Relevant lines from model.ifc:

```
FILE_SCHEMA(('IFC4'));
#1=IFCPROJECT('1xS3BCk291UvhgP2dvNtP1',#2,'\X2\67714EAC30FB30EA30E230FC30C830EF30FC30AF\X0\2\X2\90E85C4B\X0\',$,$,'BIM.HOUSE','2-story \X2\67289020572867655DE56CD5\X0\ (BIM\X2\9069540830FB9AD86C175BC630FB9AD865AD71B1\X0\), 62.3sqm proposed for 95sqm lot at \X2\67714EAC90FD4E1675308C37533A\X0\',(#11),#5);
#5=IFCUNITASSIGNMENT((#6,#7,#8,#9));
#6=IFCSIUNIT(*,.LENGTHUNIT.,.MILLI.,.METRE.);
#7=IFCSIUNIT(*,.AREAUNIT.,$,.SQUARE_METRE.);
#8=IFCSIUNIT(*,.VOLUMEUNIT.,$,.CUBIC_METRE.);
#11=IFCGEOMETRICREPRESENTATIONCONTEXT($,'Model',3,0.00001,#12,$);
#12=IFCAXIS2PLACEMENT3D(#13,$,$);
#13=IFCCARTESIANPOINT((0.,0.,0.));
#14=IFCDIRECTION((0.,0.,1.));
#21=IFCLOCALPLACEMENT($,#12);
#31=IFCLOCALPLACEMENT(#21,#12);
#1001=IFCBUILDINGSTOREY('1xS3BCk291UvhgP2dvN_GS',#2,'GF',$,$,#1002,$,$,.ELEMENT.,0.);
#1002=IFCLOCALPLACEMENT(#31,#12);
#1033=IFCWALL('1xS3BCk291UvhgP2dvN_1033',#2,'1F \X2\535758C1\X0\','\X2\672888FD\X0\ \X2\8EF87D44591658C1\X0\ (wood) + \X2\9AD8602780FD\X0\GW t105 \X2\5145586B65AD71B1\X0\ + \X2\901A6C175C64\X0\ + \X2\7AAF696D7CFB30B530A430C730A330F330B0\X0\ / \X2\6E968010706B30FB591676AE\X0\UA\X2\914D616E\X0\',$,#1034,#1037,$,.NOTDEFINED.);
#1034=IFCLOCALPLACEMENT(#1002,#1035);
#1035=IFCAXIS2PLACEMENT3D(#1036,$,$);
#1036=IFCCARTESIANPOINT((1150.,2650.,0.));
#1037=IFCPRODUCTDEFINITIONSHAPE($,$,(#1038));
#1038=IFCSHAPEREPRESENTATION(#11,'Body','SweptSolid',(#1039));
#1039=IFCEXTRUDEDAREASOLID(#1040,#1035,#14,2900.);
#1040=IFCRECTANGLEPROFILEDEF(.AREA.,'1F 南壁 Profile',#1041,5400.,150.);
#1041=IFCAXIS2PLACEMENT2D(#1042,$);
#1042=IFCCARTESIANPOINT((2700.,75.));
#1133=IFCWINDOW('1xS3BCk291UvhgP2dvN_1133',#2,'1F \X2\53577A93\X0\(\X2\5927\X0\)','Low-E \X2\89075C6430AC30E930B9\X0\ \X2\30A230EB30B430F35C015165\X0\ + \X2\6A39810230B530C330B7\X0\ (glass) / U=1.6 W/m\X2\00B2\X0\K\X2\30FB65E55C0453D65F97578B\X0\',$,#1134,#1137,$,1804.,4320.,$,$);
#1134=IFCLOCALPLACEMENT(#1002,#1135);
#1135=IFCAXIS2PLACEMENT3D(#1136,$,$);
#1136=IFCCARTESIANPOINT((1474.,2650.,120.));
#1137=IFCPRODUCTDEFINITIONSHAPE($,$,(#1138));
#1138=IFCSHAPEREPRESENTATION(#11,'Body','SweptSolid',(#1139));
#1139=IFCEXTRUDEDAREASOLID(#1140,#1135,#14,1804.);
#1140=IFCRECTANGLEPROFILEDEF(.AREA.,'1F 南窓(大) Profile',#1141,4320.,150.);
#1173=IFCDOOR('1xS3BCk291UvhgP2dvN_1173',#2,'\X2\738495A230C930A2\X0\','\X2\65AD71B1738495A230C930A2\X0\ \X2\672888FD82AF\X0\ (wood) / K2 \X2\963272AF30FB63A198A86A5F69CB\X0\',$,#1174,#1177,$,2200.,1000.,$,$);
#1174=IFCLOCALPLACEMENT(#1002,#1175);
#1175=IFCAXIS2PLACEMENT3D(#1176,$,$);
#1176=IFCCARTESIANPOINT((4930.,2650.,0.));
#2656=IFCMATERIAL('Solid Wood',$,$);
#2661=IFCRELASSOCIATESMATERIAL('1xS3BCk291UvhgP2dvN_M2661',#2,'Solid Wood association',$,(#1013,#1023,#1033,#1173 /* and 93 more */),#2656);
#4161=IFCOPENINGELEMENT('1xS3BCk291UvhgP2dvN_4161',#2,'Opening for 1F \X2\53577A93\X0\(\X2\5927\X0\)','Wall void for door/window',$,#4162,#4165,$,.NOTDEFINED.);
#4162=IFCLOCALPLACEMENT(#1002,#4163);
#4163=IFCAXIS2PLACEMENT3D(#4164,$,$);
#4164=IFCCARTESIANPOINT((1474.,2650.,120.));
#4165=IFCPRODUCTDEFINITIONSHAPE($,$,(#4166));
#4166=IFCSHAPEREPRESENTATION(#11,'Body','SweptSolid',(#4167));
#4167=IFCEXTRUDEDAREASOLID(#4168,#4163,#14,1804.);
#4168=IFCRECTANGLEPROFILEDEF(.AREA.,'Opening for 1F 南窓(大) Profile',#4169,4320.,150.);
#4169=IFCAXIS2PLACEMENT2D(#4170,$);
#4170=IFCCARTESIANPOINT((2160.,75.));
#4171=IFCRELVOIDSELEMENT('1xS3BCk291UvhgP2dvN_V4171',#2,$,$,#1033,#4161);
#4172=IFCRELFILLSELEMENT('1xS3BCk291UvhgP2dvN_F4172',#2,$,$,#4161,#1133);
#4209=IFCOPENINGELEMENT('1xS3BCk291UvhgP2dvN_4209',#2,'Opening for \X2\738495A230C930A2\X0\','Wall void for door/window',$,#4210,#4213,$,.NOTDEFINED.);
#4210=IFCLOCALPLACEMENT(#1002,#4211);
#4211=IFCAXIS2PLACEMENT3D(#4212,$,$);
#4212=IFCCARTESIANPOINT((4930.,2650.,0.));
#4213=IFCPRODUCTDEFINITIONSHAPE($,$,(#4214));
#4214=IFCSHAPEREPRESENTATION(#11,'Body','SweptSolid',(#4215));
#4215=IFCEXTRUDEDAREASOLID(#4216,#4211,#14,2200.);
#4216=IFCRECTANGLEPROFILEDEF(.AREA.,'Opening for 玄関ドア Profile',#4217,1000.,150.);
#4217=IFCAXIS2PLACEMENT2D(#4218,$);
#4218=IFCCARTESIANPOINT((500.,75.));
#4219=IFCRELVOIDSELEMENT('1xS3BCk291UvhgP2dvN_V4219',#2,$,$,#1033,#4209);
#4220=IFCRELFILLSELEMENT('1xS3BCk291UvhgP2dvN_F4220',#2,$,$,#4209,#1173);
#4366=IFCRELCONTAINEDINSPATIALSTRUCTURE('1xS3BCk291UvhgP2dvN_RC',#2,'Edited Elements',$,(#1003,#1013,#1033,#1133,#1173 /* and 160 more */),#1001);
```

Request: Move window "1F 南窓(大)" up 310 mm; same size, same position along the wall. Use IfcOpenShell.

```python
import numpy as np
import ifcopenshell
import ifcopenshell.api.geometry
import ifcopenshell.util.placement
import ifcopenshell.util.unit

model = ifcopenshell.open("model.ifc")
unit_scale = ifcopenshell.util.unit.calculate_unit_scale(model)

window = model.by_guid("1xS3BCk291UvhgP2dvN_1133")
opening = window.FillsVoids[0].RelatingOpeningElement
dz = 0.31 / unit_scale

shift = np.array([0.0, 0.0, dz])
# The window is not placed relative to its opening, so move both.
for product in (opening, window):
    matrix = ifcopenshell.util.placement.get_local_placement(product.ObjectPlacement)
    matrix[:3, 3] += shift
    ifcopenshell.api.geometry.edit_object_placement(model, product=product, matrix=matrix, is_si=False)

print(f"moved by {dz * unit_scale:+.3f} m")

model.write("model_rev.ifc")
```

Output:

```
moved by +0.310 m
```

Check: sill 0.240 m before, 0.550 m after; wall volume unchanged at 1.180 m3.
